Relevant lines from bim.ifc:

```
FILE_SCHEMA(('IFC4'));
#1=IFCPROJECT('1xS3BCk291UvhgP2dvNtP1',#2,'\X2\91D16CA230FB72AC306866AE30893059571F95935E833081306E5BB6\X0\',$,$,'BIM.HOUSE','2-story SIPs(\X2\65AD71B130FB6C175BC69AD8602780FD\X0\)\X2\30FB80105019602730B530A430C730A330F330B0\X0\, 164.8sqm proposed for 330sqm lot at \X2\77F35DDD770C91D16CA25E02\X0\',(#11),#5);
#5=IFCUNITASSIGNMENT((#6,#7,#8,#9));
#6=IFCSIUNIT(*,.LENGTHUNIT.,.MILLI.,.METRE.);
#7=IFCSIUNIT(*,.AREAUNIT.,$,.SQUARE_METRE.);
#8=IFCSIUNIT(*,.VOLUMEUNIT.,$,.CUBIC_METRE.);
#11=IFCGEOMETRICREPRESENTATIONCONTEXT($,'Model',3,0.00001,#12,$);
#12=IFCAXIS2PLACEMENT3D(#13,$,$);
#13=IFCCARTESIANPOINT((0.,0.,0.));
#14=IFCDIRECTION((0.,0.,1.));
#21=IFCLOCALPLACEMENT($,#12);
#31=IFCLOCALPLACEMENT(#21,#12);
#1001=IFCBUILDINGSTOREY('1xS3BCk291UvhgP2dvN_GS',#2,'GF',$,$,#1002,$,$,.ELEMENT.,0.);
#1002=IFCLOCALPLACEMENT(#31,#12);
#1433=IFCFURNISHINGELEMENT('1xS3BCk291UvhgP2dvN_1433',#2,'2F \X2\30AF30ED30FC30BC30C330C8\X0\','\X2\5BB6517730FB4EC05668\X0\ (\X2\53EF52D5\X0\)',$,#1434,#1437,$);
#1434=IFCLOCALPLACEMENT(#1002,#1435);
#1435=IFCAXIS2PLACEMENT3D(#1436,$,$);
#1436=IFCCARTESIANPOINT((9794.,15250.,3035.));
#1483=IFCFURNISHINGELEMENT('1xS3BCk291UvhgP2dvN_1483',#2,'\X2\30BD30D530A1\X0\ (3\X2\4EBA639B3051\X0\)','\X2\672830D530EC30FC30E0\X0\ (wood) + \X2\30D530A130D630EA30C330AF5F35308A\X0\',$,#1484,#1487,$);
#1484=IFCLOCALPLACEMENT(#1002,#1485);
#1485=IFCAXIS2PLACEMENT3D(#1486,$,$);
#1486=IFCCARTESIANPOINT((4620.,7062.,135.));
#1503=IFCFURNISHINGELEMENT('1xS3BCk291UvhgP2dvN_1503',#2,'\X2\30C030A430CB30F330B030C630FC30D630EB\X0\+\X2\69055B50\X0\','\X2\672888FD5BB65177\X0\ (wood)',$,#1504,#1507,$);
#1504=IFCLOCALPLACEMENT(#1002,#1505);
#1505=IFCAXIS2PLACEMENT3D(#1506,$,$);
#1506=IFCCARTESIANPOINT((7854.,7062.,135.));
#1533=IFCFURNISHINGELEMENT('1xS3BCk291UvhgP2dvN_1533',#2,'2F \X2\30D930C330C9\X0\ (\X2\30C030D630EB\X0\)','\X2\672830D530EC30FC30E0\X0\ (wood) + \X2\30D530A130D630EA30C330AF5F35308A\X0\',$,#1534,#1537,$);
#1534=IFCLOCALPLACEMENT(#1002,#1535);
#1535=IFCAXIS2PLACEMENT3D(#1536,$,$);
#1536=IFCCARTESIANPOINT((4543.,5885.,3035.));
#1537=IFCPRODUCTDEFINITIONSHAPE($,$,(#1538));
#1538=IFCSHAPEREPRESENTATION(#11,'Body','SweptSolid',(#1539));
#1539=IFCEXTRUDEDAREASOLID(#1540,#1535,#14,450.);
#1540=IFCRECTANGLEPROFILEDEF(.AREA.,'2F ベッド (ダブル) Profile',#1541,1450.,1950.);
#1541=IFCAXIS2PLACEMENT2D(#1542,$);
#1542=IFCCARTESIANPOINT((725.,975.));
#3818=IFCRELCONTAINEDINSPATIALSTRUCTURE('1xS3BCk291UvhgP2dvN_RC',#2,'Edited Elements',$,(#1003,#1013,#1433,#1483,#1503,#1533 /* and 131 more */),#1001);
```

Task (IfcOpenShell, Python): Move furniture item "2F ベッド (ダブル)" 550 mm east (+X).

```python
import ifcopenshell
import ifcopenshell.api.geometry
import ifcopenshell.util.placement

model = ifcopenshell.open("bim.ifc")

item = model.by_guid("1xS3BCk291UvhgP2dvN_1533")
matrix = ifcopenshell.util.placement.get_local_placement(item.ObjectPlacement)
matrix[0, 3] += 550.0
ifcopenshell.api.geometry.edit_object_placement(model, product=item, matrix=matrix, is_si=False)

print(ifcopenshell.util.placement.get_local_placement(item.ObjectPlacement).round(3) + 0.0)

model.write("bim-out.ifc")
```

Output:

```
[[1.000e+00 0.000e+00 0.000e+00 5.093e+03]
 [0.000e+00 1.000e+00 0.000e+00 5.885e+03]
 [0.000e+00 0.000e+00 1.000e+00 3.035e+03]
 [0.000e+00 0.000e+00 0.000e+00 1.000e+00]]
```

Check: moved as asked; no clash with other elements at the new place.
